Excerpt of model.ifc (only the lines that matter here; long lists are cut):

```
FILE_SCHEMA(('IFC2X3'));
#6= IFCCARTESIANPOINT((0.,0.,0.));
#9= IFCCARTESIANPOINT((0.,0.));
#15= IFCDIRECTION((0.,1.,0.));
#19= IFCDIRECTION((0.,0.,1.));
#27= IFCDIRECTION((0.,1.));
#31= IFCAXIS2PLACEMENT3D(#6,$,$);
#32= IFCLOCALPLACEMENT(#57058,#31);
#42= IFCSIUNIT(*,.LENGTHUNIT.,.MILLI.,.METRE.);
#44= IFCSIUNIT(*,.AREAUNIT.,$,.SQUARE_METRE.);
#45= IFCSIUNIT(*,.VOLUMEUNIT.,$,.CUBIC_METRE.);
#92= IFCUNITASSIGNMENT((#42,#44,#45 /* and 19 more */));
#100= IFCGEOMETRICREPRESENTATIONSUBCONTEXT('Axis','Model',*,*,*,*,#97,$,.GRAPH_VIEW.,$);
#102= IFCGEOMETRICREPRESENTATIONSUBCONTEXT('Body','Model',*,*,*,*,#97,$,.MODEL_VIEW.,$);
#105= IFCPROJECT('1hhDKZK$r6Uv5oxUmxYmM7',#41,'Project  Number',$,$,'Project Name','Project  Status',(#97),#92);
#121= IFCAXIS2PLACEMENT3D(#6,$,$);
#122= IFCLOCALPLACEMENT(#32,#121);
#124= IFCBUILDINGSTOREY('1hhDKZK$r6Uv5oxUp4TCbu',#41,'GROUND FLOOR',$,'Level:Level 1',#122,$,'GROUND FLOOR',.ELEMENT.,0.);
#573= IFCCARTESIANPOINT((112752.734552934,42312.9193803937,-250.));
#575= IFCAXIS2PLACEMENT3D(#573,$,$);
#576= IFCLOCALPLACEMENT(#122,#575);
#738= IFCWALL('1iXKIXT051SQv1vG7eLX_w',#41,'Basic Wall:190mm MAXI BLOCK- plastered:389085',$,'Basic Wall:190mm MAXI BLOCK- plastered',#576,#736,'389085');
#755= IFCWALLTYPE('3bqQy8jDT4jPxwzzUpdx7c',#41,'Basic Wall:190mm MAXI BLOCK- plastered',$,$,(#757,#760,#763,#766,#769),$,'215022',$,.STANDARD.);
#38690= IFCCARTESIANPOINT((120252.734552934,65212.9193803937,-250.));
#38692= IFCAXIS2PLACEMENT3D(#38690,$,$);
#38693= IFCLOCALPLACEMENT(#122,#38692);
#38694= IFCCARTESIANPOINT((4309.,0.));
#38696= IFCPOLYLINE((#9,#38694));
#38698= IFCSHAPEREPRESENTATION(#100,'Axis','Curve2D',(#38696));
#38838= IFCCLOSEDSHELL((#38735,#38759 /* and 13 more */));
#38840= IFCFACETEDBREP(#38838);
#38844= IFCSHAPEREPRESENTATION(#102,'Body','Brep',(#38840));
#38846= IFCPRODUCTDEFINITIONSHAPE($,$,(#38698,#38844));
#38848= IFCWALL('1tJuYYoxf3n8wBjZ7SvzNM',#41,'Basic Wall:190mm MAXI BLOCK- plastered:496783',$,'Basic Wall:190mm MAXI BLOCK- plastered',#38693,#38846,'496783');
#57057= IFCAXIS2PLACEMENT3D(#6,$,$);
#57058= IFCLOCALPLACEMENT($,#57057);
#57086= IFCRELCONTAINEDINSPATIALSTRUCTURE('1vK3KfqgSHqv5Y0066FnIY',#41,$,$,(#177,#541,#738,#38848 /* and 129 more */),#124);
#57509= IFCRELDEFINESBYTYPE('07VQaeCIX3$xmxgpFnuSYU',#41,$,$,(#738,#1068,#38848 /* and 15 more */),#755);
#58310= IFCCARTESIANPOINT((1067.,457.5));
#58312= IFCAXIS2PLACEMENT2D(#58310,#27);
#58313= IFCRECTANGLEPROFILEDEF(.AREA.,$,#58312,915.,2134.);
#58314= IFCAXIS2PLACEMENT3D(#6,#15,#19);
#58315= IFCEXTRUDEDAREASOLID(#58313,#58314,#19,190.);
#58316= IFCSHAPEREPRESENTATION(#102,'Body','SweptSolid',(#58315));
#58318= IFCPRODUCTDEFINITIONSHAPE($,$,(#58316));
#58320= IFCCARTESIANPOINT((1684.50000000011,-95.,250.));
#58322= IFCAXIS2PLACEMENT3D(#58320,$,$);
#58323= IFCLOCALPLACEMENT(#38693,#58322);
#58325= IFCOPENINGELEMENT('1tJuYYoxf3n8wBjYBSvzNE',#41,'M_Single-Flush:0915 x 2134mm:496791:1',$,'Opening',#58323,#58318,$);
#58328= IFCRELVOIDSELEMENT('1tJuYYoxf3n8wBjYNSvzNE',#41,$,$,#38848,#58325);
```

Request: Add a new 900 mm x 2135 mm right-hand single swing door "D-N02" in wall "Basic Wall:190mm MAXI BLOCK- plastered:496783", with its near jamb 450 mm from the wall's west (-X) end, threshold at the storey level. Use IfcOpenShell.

```python
import numpy as np
import ifcopenshell
import ifcopenshell.api.feature
import ifcopenshell.api.geometry
import ifcopenshell.api.root
import ifcopenshell.api.spatial
import ifcopenshell.api.type
import ifcopenshell.geom
import ifcopenshell.util.element
import ifcopenshell.util.placement
import ifcopenshell.util.representation
import ifcopenshell.util.shape
import ifcopenshell.util.unit

model = ifcopenshell.open("model.ifc")
unit_scale = ifcopenshell.util.unit.calculate_unit_scale(model)
settings = ifcopenshell.geom.settings()


def volume(element):
    """Net volume in cubic metres, openings subtracted."""
    shape = ifcopenshell.geom.create_shape(settings, element)
    return ifcopenshell.util.shape.get_volume(shape.geometry)


wall = model.by_guid("1tJuYYoxf3n8wBjZ7SvzNM")
storey = ifcopenshell.util.element.get_container(wall, ifc_class="IfcBuildingStorey")
context = ifcopenshell.util.representation.get_context(model, "Model", "Body", "MODEL_VIEW")
before = volume(wall)

width, height, from_end, sill = 0.9, 2.135, 0.45, 0.0  # metres

# The wall runs along its own X axis, and the end named is its -X end.
wall_shape = ifcopenshell.geom.create_shape(settings, wall)
x, y, z = ifcopenshell.util.shape.get_vertices(wall_shape.geometry).T
start = x.min() + from_end
face, thickness = float(y.min()), float(y.max() - y.min())
wall_matrix = ifcopenshell.util.placement.get_local_placement(wall.ObjectPlacement)
level = ifcopenshell.util.placement.get_local_placement(storey.ObjectPlacement)[2, 3]


def in_wall(x, y):
    """Placement at x, y metres in the wall's axes, at sill height."""
    matrix = wall_matrix.copy()
    matrix[:, 3] = wall_matrix @ np.array([x / unit_scale, y / unit_scale, 0.0, 1.0])
    matrix[2, 3] = level + sill / unit_scale
    return matrix


# Opening: a box that overshoots both wall faces by 50 mm.
opening = ifcopenshell.api.root.create_entity(model, ifc_class="IfcOpeningElement")
box = ifcopenshell.api.geometry.add_wall_representation(
    model, context=context, length=width, height=height, thickness=thickness + 0.1
)
ifcopenshell.api.geometry.assign_representation(model, product=opening, representation=box)
ifcopenshell.api.geometry.edit_object_placement(model, product=opening, matrix=in_wall(start, face - 0.05), is_si=False)
ifcopenshell.api.feature.add_feature(model, feature=opening, element=wall)

door = ifcopenshell.api.root.create_entity(model, ifc_class="IfcDoor", name="D-N02")
door.OverallWidth, door.OverallHeight = width / unit_scale, height / unit_scale
body = ifcopenshell.api.geometry.add_door_representation(
    model,
    context=context,
    overall_width=door.OverallWidth,
    overall_height=door.OverallHeight,
    operation_type="SINGLE_SWING_RIGHT",
    lining_properties={"LiningDepth": thickness / unit_scale, "ThresholdDepth": thickness / unit_scale},
)
ifcopenshell.api.geometry.assign_representation(model, product=door, representation=body)
ifcopenshell.api.spatial.assign_container(model, products=[door], relating_structure=storey)
fills = ifcopenshell.api.feature.add_filling(model, opening=opening, element=door)
fills.OwnerHistory = door.OwnerHistory  # required in IFC2X3

# IFC2X3 keeps the operation on the door style.
style = ifcopenshell.api.root.create_entity(model, ifc_class="IfcDoorStyle", name="D-N02")
style.OperationType, style.ConstructionType = "SINGLE_SWING_RIGHT", "NOTDEFINED"
style.ParameterTakesPrecedence = style.Sizeable = False
ifcopenshell.api.type.assign_type(model, related_objects=[door], relating_type=style)

# The lining spans the wall, so the door starts at the wall face.
ifcopenshell.api.geometry.edit_object_placement(model, product=door, matrix=in_wall(start, face), is_si=False)

after = volume(wall)

print(f"wall volume {before:.3f} -> {after:.3f} m3")

model.write("model_rev.ifc")
```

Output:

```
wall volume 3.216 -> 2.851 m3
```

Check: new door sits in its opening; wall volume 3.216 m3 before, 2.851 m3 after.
